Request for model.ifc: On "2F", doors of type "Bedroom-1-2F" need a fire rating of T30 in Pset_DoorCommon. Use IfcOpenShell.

First a look at what the model holds.

```python
import ifcopenshell
import ifcopenshell.util.element

model = ifcopenshell.open("model.ifc")
print(model.schema)
storey = next(s for s in model.by_type("IfcBuildingStorey") if s.Name == "2F")
doors = [e for e in ifcopenshell.util.element.get_decomposition(storey) if e.is_a("IfcDoor")]
seen = {}
for e in doors:
    element_type = ifcopenshell.util.element.get_type(e)
    key = (element_type.Name if element_type != e and element_type else None, ifcopenshell.util.element.get_pset(e, "Pset_DoorCommon", "FireRating"))
    seen[key] = seen.get(key, 0) + 1
for (name, value), count in sorted(seen.items(), key=str):
    print(count, "x", name, "|", value)
```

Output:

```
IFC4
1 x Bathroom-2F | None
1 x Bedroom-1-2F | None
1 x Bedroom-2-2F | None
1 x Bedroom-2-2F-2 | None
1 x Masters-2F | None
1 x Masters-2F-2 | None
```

```python
import ifcopenshell
import ifcopenshell.api.pset
import ifcopenshell.util.element

model = ifcopenshell.open("model.ifc")

storey = next(s for s in model.by_type("IfcBuildingStorey") if s.Name == "2F")
doors = [e for e in ifcopenshell.util.element.get_decomposition(storey) if e.is_a("IfcDoor")]

count = 0
for e in doors:
    element_type = ifcopenshell.util.element.get_type(e)
    if element_type in (None, e) or element_type.Name != "Bedroom-1-2F":
        continue
    # add_pset returns the element's existing set when there is one.
    pset = ifcopenshell.api.pset.add_pset(model, product=e, name="Pset_DoorCommon")
    ifcopenshell.api.pset.edit_pset(model, pset=pset, properties={"FireRating": "T30"})
    count += 1

print(count, "doors updated")

model.write("model_rev.ifc")
```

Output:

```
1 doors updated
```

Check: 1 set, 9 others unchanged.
